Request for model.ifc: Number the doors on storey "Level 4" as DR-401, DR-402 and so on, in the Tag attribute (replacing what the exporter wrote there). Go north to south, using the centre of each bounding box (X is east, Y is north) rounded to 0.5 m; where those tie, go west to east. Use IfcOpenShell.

First a look at what the model holds.

```python
import ifcopenshell
import ifcopenshell.util.element
import ifcopenshell.util.placement

model = ifcopenshell.open("model.ifc")
print(model.schema)
storey = next(s for s in model.by_type("IfcBuildingStorey") if s.Name == "Level 4")
doors = [e for e in ifcopenshell.util.element.get_decomposition(storey) if e.is_a("IfcDoor")]
for e in sorted(doors, key=lambda e: e.id()):
    origin = ifcopenshell.util.placement.get_local_placement(e.ObjectPlacement)[:3, 3]
    print(e.id(), e.Tag, e.Name, origin.round(2) + 0.0, sep=" | ")
```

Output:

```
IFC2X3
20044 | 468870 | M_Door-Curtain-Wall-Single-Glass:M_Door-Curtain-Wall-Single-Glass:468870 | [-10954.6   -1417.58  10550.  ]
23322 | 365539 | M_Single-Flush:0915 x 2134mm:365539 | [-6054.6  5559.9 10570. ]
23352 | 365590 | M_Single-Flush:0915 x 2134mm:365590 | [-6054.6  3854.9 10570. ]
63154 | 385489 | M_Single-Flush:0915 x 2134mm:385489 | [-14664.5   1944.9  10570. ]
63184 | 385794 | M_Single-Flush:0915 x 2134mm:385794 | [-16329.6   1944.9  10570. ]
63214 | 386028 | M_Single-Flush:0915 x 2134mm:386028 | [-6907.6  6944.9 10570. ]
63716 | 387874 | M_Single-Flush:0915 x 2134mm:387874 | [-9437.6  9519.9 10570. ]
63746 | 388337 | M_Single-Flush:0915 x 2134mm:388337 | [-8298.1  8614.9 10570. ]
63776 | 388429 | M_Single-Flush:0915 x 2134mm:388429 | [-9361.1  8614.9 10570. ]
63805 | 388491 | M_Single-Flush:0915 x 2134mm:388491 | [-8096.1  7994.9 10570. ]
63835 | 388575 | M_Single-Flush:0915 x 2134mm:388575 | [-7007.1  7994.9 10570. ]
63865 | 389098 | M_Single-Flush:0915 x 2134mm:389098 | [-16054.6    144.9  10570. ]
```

```python
import ifcopenshell
import ifcopenshell.geom
import ifcopenshell.util.element
import ifcopenshell.util.shape

model = ifcopenshell.open("model.ifc")
settings = ifcopenshell.geom.settings()
settings.set("use-world-coords", True)


def centre(element):
    shape = ifcopenshell.geom.create_shape(settings, element)
    return ifcopenshell.util.shape.get_bbox_centroid(shape.geometry)


storey = next(s for s in model.by_type("IfcBuildingStorey") if s.Name == "Level 4")
doors = [e for e in ifcopenshell.util.element.get_decomposition(storey) if e.is_a("IfcDoor")]

# Insertion points can sit at a corner or the storey origin, so sort by the geometry (in metres).
centres = {e: centre(e) for e in doors}
doors.sort(key=lambda e: (-round(centres[e][1] / 0.5), centres[e][0]))

for i, e in enumerate(doors, start=1):
    number = f"DR-4{i:02d}"
    e.Tag = number
    print(e.id(), number)

model.write("model_updated.ifc")
```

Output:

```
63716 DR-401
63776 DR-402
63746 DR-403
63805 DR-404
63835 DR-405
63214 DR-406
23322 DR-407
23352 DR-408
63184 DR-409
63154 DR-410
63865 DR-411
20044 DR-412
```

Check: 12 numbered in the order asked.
